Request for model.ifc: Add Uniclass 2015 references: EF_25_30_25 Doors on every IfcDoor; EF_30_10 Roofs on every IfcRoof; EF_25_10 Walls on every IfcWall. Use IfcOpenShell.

First a look at what the model holds.

```python
import ifcopenshell

model = ifcopenshell.open("model.ifc")
print(model.schema)
print("classifications:", [c.Name for c in model.by_type("IfcClassification")])
for ifc_class in ("IfcDoor", "IfcRoof", "IfcStair", "IfcWall", "IfcWindow"):
    print(ifc_class, len(model.by_type(ifc_class)))
```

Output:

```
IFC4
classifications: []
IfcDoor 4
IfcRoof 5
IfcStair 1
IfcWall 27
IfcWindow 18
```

```python
import ifcopenshell
import ifcopenshell.api.classification

model = ifcopenshell.open("model.ifc")

system = ifcopenshell.api.classification.add_classification(model, classification="Uniclass 2015")

codes = {
    "IfcDoor": ("EF_25_30_25", "Doors"),
    "IfcRoof": ("EF_30_10", "Roofs"),
    "IfcWall": ("EF_25_10", "Walls"),
}
for ifc_class, (code, name) in codes.items():
    products = model.by_type(ifc_class)
    ifcopenshell.api.classification.add_reference(
        model, products=products, classification=system, identification=code, name=name
    )
    print(code, len(products))

model.write("model_v2.ifc")
```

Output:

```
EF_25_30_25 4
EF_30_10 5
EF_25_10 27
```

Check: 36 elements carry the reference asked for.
